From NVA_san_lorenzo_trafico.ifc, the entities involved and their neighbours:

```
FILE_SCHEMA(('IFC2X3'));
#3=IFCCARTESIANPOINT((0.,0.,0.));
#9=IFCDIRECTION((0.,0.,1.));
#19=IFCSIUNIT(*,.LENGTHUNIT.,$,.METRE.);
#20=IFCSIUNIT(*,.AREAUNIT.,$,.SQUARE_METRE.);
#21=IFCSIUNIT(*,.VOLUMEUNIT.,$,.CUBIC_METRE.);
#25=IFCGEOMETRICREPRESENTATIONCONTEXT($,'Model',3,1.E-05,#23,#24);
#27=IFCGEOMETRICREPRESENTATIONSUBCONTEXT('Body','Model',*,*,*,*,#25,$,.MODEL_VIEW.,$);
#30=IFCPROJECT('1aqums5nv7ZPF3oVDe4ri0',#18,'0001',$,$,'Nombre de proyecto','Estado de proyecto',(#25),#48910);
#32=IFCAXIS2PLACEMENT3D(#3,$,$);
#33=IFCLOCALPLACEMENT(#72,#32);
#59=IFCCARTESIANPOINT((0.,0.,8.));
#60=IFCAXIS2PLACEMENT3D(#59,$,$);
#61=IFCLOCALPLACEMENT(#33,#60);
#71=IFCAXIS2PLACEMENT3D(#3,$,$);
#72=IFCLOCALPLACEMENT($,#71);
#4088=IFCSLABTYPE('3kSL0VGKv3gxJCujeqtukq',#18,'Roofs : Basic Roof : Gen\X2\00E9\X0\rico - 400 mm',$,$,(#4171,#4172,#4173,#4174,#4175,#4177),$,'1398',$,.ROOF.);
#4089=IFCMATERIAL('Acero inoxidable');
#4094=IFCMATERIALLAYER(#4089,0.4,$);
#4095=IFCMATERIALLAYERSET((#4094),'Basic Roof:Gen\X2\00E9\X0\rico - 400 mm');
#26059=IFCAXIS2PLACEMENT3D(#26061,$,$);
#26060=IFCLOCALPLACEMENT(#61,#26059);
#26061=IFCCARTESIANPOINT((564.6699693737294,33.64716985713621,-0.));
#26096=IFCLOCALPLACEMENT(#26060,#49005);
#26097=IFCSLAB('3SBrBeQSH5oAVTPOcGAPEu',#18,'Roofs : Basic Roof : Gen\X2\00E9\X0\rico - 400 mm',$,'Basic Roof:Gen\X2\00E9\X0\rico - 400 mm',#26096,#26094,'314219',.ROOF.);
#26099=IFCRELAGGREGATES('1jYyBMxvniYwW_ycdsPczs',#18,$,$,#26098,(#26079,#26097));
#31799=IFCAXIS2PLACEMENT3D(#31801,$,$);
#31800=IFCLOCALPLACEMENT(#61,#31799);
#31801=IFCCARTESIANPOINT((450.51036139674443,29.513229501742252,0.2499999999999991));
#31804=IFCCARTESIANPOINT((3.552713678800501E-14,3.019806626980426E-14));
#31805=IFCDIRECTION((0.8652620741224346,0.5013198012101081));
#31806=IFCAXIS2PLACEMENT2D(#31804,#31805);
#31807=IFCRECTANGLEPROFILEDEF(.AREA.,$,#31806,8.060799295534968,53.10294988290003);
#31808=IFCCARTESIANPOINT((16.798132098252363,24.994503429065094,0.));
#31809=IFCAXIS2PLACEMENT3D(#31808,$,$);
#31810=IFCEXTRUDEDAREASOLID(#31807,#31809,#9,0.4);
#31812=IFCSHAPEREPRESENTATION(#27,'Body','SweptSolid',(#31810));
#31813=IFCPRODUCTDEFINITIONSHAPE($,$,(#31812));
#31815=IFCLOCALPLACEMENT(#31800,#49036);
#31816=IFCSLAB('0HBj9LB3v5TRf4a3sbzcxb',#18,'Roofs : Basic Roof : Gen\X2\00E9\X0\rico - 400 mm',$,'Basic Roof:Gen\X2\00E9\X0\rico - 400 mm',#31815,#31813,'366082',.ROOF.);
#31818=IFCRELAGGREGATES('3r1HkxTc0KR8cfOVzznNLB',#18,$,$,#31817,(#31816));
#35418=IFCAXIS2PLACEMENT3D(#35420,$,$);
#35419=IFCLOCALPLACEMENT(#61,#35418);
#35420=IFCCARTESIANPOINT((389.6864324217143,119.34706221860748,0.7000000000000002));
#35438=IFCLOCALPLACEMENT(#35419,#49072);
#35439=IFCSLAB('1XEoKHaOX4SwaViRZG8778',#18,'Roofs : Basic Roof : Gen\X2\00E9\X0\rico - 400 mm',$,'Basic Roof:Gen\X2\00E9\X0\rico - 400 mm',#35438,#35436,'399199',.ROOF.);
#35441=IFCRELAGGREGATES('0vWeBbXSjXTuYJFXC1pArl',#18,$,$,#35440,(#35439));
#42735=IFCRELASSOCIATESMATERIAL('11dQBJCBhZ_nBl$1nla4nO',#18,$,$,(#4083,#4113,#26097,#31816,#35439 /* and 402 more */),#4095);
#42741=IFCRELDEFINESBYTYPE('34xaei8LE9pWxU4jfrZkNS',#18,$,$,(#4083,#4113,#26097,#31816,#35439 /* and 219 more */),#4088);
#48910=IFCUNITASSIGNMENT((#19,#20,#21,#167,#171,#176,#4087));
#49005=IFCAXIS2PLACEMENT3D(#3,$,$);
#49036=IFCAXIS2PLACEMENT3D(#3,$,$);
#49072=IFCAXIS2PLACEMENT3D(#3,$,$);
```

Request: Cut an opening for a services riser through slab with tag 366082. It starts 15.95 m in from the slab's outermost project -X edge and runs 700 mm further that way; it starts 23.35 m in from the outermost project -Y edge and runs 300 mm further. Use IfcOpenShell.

```python
import numpy as np
import ifcopenshell
import ifcopenshell.api.feature
import ifcopenshell.api.geometry
import ifcopenshell.api.root
import ifcopenshell.geom
import ifcopenshell.util.placement
import ifcopenshell.util.representation
import ifcopenshell.util.shape
import ifcopenshell.util.unit

model = ifcopenshell.open("NVA_san_lorenzo_trafico.ifc")
unit_scale = ifcopenshell.util.unit.calculate_unit_scale(model)
settings = ifcopenshell.geom.settings()


def volume(element):
    """Net volume in cubic metres, openings subtracted."""
    shape = ifcopenshell.geom.create_shape(settings, element)
    return ifcopenshell.util.shape.get_volume(shape.geometry)


slab = model.by_guid("0HBj9LB3v5TRf4a3sbzcxb")
before = volume(slab)

# Extent in the slab's own axes, in metres. The edges named are its -X and -Y sides.
slab_shape = ifcopenshell.geom.create_shape(settings, slab)
vertices = ifcopenshell.util.shape.get_vertices(slab_shape.geometry)
x_min, y_min, bottom = vertices.min(axis=0)
top = vertices[:, 2].max()

opening = ifcopenshell.api.root.create_entity(model, ifc_class="IfcOpeningElement", name="Services riser opening")
context = ifcopenshell.util.representation.get_context(model, "Model", "Body", "MODEL_VIEW")
width, depth = 0.7, 0.3
outline = [(0.0, 0.0), (width, 0.0), (width, depth), (0.0, depth), (0.0, 0.0)]
# Overshoot both faces by 50 mm so the cut is clean.
shape = ifcopenshell.api.geometry.add_slab_representation(
    model, context=context, depth=top - bottom + 0.1, polyline=outline
)
ifcopenshell.api.geometry.assign_representation(model, product=opening, representation=shape)

matrix = ifcopenshell.util.placement.get_local_placement(slab.ObjectPlacement)
matrix[:, 3] = matrix @ np.append(np.array([x_min + 15.95, y_min + 23.35, bottom - 0.05]) / unit_scale, 1.0)
ifcopenshell.api.geometry.edit_object_placement(model, product=opening, matrix=matrix, is_si=False)
ifcopenshell.api.feature.add_feature(model, feature=opening, element=slab)

after = volume(slab)

print(f"slab volume {before:.3f} -> {after:.3f} m3")

model.write("NVA_san_lorenzo_trafico_rev.ifc")
```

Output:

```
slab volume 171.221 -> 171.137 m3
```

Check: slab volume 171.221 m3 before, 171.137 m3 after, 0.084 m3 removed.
